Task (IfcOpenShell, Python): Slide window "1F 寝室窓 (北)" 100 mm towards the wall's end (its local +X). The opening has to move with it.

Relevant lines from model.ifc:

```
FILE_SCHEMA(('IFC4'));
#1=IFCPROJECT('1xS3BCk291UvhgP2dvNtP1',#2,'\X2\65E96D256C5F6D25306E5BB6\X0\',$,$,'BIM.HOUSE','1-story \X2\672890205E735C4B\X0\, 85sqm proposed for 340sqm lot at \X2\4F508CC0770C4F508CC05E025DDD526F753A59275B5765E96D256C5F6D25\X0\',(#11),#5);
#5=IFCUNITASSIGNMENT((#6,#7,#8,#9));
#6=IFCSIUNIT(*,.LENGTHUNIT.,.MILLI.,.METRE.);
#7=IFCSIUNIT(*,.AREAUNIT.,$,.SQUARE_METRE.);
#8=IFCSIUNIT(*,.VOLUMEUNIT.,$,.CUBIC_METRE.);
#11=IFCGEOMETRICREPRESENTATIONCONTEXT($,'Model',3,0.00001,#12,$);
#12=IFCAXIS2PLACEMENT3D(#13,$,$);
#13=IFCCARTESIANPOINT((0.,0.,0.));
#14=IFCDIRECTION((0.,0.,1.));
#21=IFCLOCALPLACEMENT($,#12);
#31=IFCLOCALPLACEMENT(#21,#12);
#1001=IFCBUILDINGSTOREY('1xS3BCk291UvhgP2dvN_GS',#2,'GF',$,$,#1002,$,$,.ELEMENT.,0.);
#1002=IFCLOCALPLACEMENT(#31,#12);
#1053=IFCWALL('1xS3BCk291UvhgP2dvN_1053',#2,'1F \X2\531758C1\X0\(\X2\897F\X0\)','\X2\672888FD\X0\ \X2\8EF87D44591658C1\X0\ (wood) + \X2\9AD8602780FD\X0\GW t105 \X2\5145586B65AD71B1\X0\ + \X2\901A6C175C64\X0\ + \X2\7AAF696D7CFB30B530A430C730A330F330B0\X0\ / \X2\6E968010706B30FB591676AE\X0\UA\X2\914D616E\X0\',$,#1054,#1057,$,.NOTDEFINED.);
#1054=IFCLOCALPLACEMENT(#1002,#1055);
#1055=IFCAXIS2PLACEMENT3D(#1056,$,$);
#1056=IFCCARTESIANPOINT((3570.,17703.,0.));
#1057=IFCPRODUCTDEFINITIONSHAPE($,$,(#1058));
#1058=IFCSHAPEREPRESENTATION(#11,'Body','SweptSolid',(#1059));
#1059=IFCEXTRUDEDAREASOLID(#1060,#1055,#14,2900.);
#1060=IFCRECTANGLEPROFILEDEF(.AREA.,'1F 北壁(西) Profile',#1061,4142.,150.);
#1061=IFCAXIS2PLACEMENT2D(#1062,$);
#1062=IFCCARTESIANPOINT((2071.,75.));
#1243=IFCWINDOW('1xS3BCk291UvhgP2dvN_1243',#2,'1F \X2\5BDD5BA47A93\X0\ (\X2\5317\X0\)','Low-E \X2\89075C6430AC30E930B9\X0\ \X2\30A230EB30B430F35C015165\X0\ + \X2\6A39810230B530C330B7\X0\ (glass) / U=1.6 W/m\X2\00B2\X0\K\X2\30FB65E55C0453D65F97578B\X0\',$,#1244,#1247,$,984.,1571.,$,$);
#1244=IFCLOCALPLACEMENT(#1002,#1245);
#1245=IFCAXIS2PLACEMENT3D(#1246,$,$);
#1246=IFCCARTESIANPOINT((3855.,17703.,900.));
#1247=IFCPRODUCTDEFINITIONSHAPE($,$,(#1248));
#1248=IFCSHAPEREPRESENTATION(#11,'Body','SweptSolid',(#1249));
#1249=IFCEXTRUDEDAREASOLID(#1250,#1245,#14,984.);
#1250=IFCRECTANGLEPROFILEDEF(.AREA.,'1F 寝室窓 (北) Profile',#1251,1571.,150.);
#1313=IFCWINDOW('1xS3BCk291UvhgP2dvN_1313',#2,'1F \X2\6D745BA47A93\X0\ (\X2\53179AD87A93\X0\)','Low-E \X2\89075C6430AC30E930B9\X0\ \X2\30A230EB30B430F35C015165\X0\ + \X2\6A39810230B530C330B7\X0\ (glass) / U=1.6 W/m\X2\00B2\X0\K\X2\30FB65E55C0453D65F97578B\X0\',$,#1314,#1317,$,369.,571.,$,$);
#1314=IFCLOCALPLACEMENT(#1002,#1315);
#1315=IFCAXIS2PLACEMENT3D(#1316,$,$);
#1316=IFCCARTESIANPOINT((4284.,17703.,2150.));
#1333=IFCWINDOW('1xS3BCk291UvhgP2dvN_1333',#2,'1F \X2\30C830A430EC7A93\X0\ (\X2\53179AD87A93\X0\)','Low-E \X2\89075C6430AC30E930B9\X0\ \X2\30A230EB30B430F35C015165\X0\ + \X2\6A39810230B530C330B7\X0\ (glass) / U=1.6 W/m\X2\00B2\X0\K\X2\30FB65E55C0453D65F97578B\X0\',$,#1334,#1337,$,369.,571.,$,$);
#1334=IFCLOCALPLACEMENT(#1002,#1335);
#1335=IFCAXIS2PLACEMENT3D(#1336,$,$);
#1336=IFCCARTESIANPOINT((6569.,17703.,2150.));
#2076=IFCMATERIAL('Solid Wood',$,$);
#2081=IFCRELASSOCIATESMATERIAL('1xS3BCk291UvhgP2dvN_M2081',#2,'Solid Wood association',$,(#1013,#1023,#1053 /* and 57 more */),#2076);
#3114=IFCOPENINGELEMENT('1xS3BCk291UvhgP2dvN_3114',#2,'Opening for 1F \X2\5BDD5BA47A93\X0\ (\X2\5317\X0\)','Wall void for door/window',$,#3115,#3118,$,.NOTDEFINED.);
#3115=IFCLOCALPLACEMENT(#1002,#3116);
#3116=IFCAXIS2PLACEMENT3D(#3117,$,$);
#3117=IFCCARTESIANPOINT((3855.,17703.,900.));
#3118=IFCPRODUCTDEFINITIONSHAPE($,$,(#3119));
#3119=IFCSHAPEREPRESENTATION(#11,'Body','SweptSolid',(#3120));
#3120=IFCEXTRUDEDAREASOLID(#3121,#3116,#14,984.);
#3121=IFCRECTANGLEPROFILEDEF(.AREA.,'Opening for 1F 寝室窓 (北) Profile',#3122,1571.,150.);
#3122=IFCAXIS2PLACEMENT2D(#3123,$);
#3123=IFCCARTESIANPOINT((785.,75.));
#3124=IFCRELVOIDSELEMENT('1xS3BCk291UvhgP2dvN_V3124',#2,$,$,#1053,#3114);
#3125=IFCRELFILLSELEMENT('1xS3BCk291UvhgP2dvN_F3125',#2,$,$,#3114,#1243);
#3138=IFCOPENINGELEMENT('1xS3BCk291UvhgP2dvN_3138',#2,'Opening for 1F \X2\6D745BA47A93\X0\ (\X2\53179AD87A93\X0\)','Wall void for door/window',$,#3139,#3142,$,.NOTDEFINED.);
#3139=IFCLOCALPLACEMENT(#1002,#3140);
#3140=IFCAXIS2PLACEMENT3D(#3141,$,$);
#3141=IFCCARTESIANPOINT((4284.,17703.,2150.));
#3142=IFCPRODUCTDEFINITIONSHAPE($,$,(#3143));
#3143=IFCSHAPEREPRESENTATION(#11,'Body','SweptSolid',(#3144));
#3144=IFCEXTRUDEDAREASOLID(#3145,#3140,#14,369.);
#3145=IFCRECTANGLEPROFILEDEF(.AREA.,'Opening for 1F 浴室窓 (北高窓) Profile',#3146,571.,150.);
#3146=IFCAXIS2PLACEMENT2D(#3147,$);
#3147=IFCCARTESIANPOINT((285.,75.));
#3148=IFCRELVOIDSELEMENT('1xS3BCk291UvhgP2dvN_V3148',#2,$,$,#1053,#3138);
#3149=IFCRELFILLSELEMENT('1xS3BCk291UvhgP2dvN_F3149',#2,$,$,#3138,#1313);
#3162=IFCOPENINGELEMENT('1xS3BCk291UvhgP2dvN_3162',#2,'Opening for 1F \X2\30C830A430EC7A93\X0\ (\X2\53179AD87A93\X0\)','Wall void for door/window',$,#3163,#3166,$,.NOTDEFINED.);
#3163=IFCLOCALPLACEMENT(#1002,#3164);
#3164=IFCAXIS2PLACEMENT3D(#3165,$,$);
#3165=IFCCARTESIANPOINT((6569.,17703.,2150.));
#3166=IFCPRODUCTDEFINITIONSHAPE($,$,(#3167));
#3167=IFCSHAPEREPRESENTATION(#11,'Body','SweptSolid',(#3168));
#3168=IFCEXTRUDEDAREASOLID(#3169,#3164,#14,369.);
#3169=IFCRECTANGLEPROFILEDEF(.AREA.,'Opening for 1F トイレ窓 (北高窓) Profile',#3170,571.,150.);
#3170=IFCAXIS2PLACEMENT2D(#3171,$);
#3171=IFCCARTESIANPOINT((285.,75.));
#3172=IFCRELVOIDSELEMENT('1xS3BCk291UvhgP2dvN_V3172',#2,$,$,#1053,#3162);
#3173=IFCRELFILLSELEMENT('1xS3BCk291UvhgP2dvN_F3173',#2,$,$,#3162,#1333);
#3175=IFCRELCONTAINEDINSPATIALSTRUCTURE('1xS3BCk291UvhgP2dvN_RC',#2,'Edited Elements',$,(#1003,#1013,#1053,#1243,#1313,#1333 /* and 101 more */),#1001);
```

```python
import ifcopenshell
import ifcopenshell.api.geometry
import ifcopenshell.util.placement
import ifcopenshell.util.unit

model = ifcopenshell.open("model.ifc")
unit_scale = ifcopenshell.util.unit.calculate_unit_scale(model)

window = model.by_guid("1xS3BCk291UvhgP2dvN_1243")
opening = window.FillsVoids[0].RelatingOpeningElement
wall = opening.VoidsElements[0].RelatingBuildingElement

wall_matrix = ifcopenshell.util.placement.get_local_placement(wall.ObjectPlacement)
shift = wall_matrix[:3, 0] * 0.1 / unit_scale
before = ifcopenshell.util.placement.get_local_placement(window.ObjectPlacement)[:3, 3].copy()

# The window is not placed relative to its opening, so move both.
for product in (opening, window):
    matrix = ifcopenshell.util.placement.get_local_placement(product.ObjectPlacement)
    matrix[:3, 3] += shift
    ifcopenshell.api.geometry.edit_object_placement(model, product=product, matrix=matrix, is_si=False)

after = ifcopenshell.util.placement.get_local_placement(window.ObjectPlacement)[:3, 3]
print("window moved by", (after - before).round(3) + 0.0)

model.write("model-out.ifc")
```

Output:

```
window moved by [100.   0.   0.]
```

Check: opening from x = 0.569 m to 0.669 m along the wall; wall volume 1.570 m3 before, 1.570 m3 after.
